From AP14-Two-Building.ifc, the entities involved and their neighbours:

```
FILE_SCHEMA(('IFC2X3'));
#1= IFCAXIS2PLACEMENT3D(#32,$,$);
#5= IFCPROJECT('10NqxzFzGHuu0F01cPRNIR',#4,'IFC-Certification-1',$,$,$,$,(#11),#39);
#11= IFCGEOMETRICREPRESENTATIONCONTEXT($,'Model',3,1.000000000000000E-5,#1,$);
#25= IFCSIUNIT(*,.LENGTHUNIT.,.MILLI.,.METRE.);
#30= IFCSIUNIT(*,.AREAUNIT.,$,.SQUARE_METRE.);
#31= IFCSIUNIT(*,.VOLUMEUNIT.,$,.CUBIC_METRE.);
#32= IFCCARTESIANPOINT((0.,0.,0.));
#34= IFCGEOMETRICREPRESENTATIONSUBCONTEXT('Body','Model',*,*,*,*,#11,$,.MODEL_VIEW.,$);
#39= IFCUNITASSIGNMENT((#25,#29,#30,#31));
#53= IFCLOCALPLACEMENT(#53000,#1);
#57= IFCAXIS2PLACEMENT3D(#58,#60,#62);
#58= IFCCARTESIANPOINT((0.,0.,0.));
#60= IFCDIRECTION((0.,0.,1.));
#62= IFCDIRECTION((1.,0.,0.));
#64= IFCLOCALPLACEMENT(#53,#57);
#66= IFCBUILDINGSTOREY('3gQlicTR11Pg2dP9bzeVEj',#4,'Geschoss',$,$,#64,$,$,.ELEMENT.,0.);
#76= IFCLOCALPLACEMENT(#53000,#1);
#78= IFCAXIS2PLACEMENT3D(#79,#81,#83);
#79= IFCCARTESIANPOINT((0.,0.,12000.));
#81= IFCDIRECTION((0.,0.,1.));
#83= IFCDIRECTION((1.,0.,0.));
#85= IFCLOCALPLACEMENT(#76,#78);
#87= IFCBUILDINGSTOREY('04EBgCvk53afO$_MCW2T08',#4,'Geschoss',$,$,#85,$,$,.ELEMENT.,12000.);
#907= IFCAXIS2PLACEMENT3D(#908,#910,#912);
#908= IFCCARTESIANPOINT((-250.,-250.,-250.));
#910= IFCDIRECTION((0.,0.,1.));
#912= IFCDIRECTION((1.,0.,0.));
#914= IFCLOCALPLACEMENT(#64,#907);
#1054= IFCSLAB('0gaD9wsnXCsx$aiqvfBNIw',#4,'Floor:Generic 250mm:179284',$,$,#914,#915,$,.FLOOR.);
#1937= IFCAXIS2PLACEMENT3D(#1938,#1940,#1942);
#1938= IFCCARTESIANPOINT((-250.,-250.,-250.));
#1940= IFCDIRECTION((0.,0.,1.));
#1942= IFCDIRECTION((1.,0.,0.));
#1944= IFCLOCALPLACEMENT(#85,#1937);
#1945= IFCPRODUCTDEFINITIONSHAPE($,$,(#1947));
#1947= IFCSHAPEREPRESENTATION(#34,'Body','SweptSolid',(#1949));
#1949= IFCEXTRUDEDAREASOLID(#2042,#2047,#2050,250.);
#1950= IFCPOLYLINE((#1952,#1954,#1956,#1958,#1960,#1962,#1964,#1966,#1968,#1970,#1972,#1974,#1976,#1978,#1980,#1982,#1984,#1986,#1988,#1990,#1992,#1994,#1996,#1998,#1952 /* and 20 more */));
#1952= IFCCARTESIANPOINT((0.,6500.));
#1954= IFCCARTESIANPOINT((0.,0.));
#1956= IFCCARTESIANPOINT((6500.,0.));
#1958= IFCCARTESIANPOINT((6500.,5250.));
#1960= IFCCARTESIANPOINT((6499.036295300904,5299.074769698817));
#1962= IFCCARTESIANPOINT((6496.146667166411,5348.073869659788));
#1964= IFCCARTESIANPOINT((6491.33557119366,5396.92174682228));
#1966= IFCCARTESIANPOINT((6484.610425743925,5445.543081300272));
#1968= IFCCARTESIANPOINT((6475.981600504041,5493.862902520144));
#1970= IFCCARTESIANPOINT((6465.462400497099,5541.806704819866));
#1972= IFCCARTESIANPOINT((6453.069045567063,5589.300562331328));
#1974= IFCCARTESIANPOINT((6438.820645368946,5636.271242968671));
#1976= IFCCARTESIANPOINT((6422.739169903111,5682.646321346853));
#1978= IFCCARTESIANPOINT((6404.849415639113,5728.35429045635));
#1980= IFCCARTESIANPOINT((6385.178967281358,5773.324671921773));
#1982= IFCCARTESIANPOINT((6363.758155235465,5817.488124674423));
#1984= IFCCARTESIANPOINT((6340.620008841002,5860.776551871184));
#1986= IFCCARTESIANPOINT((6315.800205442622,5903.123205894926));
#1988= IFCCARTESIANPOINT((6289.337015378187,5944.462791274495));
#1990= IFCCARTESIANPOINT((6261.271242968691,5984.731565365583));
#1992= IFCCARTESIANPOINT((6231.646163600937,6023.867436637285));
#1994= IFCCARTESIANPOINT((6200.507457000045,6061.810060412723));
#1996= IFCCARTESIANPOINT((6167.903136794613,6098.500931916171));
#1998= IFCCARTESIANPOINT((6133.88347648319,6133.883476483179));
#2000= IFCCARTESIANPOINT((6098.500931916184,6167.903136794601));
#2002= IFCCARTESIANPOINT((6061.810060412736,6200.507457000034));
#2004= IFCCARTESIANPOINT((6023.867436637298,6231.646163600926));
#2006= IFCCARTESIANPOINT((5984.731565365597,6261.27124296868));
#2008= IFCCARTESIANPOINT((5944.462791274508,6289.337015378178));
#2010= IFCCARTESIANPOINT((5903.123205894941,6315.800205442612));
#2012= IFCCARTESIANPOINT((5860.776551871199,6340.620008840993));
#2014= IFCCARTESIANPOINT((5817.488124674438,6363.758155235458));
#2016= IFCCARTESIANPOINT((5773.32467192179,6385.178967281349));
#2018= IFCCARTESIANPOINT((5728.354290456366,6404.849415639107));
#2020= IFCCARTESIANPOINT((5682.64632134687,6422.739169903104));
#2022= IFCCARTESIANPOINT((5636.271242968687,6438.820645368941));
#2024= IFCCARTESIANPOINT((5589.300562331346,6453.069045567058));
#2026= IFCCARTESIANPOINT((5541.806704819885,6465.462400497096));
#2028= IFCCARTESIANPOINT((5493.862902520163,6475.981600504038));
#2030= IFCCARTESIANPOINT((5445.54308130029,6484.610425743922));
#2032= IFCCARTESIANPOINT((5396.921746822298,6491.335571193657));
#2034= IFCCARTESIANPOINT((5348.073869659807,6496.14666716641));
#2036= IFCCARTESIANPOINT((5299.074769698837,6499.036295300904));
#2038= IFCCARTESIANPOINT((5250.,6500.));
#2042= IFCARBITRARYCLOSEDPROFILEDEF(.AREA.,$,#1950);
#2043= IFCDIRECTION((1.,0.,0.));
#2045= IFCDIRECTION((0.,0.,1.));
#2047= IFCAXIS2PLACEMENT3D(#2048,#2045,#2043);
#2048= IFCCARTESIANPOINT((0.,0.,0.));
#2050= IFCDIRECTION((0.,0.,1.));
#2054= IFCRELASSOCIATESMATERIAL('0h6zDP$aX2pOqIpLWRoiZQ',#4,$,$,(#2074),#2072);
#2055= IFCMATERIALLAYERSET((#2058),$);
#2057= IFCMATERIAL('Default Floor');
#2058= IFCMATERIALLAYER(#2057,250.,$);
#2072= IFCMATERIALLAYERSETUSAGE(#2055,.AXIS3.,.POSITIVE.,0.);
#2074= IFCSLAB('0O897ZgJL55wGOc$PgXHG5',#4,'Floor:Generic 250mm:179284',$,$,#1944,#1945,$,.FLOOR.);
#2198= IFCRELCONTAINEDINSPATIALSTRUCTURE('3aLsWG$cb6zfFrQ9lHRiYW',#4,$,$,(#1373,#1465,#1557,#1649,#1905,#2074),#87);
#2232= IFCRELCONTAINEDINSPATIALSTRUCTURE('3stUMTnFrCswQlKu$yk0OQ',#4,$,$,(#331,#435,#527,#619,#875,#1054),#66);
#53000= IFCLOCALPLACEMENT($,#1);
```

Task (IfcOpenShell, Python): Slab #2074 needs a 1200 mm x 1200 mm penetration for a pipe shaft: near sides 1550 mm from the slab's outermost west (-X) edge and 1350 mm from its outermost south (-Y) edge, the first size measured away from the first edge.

```python
import numpy as np
import ifcopenshell
import ifcopenshell.api.feature
import ifcopenshell.api.geometry
import ifcopenshell.api.root
import ifcopenshell.geom
import ifcopenshell.util.placement
import ifcopenshell.util.representation
import ifcopenshell.util.shape
import ifcopenshell.util.unit

model = ifcopenshell.open("AP14-Two-Building.ifc")
unit_scale = ifcopenshell.util.unit.calculate_unit_scale(model)
settings = ifcopenshell.geom.settings()


def volume(element):
    """Net volume in cubic metres, openings subtracted."""
    shape = ifcopenshell.geom.create_shape(settings, element)
    return ifcopenshell.util.shape.get_volume(shape.geometry)


slab = model.by_id(2074)
before = volume(slab)

# Extent in the slab's own axes, in metres. The edges named are its -X and -Y sides.
slab_shape = ifcopenshell.geom.create_shape(settings, slab)
vertices = ifcopenshell.util.shape.get_vertices(slab_shape.geometry)
x_min, y_min, bottom = vertices.min(axis=0)
top = vertices[:, 2].max()

opening = ifcopenshell.api.root.create_entity(model, ifc_class="IfcOpeningElement", name="Pipe shaft opening")
context = ifcopenshell.util.representation.get_context(model, "Model", "Body", "MODEL_VIEW")
width, depth = 1.2, 1.2
outline = [(0.0, 0.0), (width, 0.0), (width, depth), (0.0, depth), (0.0, 0.0)]
# Overshoot both faces by 50 mm so the cut is clean.
shape = ifcopenshell.api.geometry.add_slab_representation(
    model, context=context, depth=top - bottom + 0.1, polyline=outline
)
ifcopenshell.api.geometry.assign_representation(model, product=opening, representation=shape)

matrix = ifcopenshell.util.placement.get_local_placement(slab.ObjectPlacement)
matrix[:, 3] = matrix @ np.append(np.array([x_min + 1.55, y_min + 1.35, bottom - 0.05]) / unit_scale, 1.0)
ifcopenshell.api.geometry.edit_object_placement(model, product=opening, matrix=matrix, is_si=False)
ifcopenshell.api.feature.add_feature(model, feature=opening, element=slab)

after = volume(slab)

print(f"slab volume {before:.3f} -> {after:.3f} m3")

model.write("AP14-Two-Building_edited.ifc")
```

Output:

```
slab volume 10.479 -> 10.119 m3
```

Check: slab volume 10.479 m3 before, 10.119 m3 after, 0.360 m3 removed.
